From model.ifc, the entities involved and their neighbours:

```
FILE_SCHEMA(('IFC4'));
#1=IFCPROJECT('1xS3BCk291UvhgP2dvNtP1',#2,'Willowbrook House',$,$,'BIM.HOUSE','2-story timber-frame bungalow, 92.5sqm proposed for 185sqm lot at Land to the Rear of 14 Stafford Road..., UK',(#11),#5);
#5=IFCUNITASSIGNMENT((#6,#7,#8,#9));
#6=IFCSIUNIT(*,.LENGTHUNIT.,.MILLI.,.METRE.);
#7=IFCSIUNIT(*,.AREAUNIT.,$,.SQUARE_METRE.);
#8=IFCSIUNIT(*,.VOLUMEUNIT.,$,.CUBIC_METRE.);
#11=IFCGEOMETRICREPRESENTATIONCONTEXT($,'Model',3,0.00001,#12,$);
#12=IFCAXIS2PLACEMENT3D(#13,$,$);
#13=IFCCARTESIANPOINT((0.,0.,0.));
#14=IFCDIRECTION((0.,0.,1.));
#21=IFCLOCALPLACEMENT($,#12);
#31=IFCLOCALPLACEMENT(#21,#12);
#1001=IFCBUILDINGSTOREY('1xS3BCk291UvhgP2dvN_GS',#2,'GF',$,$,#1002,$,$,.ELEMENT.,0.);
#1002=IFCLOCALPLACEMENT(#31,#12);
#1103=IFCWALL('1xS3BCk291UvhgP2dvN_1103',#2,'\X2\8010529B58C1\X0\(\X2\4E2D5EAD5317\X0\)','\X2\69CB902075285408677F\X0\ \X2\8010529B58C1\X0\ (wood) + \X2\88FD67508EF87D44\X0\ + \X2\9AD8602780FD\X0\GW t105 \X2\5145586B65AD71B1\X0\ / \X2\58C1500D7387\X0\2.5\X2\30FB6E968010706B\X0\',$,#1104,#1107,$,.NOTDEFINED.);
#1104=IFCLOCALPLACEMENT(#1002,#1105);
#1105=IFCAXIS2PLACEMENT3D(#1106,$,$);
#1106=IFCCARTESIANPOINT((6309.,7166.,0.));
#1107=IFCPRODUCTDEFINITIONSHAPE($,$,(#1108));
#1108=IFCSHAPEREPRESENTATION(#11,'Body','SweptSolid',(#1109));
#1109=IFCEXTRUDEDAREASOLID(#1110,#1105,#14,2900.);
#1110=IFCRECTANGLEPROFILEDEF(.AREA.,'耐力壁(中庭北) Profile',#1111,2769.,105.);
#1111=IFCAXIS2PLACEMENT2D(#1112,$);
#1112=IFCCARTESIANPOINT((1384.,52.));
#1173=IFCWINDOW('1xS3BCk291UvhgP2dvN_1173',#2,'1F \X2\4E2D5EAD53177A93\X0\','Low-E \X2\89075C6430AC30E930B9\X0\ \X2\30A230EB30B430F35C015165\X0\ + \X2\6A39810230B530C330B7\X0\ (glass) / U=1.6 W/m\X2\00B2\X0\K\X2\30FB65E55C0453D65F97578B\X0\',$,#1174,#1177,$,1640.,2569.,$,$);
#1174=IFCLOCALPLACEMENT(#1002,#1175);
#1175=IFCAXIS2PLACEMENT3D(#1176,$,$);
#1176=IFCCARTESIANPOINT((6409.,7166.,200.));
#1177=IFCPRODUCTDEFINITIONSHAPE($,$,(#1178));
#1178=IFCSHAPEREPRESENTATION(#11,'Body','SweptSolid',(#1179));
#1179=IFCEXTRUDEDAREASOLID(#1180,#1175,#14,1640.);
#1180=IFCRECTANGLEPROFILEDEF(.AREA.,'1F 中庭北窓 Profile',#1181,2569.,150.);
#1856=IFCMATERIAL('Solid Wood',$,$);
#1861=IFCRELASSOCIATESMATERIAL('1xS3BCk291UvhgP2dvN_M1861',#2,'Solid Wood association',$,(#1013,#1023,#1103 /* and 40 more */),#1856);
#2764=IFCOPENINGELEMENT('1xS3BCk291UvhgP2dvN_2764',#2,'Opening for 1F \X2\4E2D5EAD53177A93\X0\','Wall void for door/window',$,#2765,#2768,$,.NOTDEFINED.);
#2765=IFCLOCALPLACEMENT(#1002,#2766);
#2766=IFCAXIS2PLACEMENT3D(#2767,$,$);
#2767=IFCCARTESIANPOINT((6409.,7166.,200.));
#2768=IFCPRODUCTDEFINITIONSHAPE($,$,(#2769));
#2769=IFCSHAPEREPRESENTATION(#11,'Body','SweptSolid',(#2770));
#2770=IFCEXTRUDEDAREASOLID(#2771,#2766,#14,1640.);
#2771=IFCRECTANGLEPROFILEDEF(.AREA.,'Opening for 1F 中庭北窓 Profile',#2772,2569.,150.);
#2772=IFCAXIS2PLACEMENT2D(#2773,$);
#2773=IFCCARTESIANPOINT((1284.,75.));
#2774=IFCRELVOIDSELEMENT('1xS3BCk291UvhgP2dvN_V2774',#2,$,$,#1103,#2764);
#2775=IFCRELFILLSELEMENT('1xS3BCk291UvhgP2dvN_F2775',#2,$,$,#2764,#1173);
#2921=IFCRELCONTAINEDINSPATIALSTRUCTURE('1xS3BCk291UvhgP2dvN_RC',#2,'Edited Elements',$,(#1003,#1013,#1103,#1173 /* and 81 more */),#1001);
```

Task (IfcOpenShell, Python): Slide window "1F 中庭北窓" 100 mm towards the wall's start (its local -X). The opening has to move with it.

```python
import ifcopenshell
import ifcopenshell.api.geometry
import ifcopenshell.util.placement
import ifcopenshell.util.unit

model = ifcopenshell.open("model.ifc")
unit_scale = ifcopenshell.util.unit.calculate_unit_scale(model)

window = model.by_id(1173)
opening = window.FillsVoids[0].RelatingOpeningElement
wall = opening.VoidsElements[0].RelatingBuildingElement

wall_matrix = ifcopenshell.util.placement.get_local_placement(wall.ObjectPlacement)
shift = wall_matrix[:3, 0] * -0.1 / unit_scale
before = ifcopenshell.util.placement.get_local_placement(window.ObjectPlacement)[:3, 3].copy()

# The window is not placed relative to its opening, so move both.
for product in (opening, window):
    matrix = ifcopenshell.util.placement.get_local_placement(product.ObjectPlacement)
    matrix[:3, 3] += shift
    ifcopenshell.api.geometry.edit_object_placement(model, product=product, matrix=matrix, is_si=False)

after = ifcopenshell.util.placement.get_local_placement(window.ObjectPlacement)[:3, 3]
print("window moved by", (after - before).round(3) + 0.0)

model.write("model_updated.ifc")
```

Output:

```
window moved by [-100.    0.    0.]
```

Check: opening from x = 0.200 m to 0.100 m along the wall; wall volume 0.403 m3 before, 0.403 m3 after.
